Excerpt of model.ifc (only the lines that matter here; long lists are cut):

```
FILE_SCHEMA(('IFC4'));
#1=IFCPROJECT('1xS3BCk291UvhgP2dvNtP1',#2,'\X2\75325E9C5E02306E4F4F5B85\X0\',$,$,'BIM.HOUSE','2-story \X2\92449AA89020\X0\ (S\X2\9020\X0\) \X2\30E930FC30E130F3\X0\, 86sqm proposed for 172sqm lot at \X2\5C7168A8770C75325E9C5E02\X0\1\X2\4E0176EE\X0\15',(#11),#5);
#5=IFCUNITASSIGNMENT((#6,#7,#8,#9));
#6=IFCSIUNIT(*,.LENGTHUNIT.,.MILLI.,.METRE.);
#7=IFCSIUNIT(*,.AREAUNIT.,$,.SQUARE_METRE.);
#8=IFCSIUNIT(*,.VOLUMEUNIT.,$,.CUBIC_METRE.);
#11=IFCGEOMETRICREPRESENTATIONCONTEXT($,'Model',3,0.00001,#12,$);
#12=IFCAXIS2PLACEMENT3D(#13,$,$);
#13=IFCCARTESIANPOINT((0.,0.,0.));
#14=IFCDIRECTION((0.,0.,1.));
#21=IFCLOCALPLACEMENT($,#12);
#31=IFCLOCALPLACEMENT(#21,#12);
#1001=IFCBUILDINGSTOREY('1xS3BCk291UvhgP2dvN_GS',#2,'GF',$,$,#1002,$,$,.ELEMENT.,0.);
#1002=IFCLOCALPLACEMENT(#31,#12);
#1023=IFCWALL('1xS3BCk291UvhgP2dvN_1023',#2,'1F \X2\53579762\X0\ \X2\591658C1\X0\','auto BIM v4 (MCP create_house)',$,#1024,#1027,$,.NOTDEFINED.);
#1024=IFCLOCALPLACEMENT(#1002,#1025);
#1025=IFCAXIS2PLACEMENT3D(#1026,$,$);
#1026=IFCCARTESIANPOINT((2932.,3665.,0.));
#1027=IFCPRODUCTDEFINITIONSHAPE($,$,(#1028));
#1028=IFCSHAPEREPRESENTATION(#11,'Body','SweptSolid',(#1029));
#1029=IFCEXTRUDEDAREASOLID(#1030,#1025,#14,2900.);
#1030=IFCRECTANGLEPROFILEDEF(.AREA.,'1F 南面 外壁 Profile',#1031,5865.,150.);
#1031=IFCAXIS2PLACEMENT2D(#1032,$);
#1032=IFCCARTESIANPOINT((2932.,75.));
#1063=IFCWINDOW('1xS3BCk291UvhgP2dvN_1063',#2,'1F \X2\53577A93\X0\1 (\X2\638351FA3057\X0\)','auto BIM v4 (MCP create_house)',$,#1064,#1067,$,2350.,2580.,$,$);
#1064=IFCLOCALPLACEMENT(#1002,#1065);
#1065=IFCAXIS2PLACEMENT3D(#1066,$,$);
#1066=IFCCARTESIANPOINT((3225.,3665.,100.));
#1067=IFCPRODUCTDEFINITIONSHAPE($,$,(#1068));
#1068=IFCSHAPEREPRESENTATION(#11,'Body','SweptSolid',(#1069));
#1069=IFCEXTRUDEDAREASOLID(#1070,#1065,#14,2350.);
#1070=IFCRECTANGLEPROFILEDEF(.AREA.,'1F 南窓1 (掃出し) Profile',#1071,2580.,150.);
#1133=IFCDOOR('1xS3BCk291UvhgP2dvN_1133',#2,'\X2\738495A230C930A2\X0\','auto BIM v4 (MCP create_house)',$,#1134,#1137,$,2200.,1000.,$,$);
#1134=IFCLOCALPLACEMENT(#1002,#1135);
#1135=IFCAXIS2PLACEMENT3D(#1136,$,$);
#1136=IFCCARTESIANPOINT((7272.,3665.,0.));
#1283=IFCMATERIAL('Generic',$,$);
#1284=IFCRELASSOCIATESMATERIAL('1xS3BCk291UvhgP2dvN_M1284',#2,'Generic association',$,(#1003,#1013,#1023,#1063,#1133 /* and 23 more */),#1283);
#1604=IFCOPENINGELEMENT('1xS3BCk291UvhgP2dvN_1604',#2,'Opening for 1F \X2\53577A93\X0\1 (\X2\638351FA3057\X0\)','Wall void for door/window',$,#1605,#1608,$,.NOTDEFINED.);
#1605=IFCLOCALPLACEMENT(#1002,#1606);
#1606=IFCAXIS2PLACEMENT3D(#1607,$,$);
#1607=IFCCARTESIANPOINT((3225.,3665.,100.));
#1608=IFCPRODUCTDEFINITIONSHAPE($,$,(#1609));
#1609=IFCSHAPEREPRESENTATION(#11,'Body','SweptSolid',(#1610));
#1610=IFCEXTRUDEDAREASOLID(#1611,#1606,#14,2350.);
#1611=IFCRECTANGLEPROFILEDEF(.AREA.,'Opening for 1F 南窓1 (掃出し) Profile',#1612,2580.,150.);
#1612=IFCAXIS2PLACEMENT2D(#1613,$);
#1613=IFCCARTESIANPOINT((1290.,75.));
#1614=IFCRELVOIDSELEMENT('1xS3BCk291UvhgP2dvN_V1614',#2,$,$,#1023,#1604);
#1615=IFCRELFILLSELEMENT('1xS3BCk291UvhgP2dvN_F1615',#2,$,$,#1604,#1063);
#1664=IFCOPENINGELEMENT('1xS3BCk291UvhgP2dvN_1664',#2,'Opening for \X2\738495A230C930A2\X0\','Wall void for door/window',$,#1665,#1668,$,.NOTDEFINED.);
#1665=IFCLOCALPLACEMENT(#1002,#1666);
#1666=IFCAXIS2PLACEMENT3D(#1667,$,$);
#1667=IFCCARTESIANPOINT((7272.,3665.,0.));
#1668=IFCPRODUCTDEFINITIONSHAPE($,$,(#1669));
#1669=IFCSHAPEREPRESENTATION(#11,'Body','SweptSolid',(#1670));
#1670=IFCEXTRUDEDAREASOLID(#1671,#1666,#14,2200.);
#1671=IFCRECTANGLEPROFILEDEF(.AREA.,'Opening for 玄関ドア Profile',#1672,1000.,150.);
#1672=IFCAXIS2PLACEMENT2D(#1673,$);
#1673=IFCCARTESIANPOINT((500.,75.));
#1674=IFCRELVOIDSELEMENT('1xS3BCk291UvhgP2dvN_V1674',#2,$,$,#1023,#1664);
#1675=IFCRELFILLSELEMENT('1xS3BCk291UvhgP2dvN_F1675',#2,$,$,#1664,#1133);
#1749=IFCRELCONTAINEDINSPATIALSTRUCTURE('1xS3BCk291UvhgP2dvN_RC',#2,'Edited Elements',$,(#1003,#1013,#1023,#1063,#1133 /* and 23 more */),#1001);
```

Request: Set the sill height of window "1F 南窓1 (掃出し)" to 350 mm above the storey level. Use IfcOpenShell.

```python
import numpy as np
import ifcopenshell
import ifcopenshell.api.geometry
import ifcopenshell.geom
import ifcopenshell.util.element
import ifcopenshell.util.placement
import ifcopenshell.util.shape
import ifcopenshell.util.unit

model = ifcopenshell.open("model.ifc")
unit_scale = ifcopenshell.util.unit.calculate_unit_scale(model)

window = model.by_guid("1xS3BCk291UvhgP2dvN_1063")
opening = window.FillsVoids[0].RelatingOpeningElement
storey = ifcopenshell.util.element.get_container(window, ifc_class="IfcBuildingStorey")
level = ifcopenshell.util.placement.get_local_placement(storey.ObjectPlacement)[2, 3]

# The opening's origin need not be at the sill, so measure its lowest point.
shape = ifcopenshell.geom.create_shape(ifcopenshell.geom.settings(), opening)
bottom = ifcopenshell.util.shape.get_shape_bottom_elevation(shape, shape.geometry) / unit_scale
dz = level + 0.35 / unit_scale - bottom

shift = np.array([0.0, 0.0, dz])
# The window is not placed relative to its opening, so move both.
for product in (opening, window):
    matrix = ifcopenshell.util.placement.get_local_placement(product.ObjectPlacement)
    matrix[:3, 3] += shift
    ifcopenshell.api.geometry.edit_object_placement(model, product=product, matrix=matrix, is_si=False)

print(f"moved by {dz * unit_scale:+.3f} m")

model.write("model-out.ifc")
```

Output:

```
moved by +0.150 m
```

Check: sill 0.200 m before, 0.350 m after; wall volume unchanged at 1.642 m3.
